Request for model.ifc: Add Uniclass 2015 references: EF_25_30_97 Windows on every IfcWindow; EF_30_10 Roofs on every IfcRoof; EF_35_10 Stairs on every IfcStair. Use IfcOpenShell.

First a look at what the model holds.

```python
import ifcopenshell

model = ifcopenshell.open("model.ifc")
print(model.schema)
print("classifications:", [c.Name for c in model.by_type("IfcClassification")])
for ifc_class in ("IfcDoor", "IfcRoof", "IfcStair", "IfcWall", "IfcWindow"):
    print(ifc_class, len(model.by_type(ifc_class)))
```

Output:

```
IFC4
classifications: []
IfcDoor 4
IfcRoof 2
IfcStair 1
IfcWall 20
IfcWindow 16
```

```python
import ifcopenshell
import ifcopenshell.api.classification

model = ifcopenshell.open("model.ifc")

system = ifcopenshell.api.classification.add_classification(model, classification="Uniclass 2015")

codes = {
    "IfcWindow": ("EF_25_30_97", "Windows"),
    "IfcRoof": ("EF_30_10", "Roofs"),
    "IfcStair": ("EF_35_10", "Stairs"),
}
for ifc_class, (code, name) in codes.items():
    products = model.by_type(ifc_class)
    ifcopenshell.api.classification.add_reference(
        model, products=products, classification=system, identification=code, name=name
    )
    print(code, len(products))

model.write("model_rev.ifc")
```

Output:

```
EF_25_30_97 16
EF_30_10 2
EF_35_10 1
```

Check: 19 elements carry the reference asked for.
